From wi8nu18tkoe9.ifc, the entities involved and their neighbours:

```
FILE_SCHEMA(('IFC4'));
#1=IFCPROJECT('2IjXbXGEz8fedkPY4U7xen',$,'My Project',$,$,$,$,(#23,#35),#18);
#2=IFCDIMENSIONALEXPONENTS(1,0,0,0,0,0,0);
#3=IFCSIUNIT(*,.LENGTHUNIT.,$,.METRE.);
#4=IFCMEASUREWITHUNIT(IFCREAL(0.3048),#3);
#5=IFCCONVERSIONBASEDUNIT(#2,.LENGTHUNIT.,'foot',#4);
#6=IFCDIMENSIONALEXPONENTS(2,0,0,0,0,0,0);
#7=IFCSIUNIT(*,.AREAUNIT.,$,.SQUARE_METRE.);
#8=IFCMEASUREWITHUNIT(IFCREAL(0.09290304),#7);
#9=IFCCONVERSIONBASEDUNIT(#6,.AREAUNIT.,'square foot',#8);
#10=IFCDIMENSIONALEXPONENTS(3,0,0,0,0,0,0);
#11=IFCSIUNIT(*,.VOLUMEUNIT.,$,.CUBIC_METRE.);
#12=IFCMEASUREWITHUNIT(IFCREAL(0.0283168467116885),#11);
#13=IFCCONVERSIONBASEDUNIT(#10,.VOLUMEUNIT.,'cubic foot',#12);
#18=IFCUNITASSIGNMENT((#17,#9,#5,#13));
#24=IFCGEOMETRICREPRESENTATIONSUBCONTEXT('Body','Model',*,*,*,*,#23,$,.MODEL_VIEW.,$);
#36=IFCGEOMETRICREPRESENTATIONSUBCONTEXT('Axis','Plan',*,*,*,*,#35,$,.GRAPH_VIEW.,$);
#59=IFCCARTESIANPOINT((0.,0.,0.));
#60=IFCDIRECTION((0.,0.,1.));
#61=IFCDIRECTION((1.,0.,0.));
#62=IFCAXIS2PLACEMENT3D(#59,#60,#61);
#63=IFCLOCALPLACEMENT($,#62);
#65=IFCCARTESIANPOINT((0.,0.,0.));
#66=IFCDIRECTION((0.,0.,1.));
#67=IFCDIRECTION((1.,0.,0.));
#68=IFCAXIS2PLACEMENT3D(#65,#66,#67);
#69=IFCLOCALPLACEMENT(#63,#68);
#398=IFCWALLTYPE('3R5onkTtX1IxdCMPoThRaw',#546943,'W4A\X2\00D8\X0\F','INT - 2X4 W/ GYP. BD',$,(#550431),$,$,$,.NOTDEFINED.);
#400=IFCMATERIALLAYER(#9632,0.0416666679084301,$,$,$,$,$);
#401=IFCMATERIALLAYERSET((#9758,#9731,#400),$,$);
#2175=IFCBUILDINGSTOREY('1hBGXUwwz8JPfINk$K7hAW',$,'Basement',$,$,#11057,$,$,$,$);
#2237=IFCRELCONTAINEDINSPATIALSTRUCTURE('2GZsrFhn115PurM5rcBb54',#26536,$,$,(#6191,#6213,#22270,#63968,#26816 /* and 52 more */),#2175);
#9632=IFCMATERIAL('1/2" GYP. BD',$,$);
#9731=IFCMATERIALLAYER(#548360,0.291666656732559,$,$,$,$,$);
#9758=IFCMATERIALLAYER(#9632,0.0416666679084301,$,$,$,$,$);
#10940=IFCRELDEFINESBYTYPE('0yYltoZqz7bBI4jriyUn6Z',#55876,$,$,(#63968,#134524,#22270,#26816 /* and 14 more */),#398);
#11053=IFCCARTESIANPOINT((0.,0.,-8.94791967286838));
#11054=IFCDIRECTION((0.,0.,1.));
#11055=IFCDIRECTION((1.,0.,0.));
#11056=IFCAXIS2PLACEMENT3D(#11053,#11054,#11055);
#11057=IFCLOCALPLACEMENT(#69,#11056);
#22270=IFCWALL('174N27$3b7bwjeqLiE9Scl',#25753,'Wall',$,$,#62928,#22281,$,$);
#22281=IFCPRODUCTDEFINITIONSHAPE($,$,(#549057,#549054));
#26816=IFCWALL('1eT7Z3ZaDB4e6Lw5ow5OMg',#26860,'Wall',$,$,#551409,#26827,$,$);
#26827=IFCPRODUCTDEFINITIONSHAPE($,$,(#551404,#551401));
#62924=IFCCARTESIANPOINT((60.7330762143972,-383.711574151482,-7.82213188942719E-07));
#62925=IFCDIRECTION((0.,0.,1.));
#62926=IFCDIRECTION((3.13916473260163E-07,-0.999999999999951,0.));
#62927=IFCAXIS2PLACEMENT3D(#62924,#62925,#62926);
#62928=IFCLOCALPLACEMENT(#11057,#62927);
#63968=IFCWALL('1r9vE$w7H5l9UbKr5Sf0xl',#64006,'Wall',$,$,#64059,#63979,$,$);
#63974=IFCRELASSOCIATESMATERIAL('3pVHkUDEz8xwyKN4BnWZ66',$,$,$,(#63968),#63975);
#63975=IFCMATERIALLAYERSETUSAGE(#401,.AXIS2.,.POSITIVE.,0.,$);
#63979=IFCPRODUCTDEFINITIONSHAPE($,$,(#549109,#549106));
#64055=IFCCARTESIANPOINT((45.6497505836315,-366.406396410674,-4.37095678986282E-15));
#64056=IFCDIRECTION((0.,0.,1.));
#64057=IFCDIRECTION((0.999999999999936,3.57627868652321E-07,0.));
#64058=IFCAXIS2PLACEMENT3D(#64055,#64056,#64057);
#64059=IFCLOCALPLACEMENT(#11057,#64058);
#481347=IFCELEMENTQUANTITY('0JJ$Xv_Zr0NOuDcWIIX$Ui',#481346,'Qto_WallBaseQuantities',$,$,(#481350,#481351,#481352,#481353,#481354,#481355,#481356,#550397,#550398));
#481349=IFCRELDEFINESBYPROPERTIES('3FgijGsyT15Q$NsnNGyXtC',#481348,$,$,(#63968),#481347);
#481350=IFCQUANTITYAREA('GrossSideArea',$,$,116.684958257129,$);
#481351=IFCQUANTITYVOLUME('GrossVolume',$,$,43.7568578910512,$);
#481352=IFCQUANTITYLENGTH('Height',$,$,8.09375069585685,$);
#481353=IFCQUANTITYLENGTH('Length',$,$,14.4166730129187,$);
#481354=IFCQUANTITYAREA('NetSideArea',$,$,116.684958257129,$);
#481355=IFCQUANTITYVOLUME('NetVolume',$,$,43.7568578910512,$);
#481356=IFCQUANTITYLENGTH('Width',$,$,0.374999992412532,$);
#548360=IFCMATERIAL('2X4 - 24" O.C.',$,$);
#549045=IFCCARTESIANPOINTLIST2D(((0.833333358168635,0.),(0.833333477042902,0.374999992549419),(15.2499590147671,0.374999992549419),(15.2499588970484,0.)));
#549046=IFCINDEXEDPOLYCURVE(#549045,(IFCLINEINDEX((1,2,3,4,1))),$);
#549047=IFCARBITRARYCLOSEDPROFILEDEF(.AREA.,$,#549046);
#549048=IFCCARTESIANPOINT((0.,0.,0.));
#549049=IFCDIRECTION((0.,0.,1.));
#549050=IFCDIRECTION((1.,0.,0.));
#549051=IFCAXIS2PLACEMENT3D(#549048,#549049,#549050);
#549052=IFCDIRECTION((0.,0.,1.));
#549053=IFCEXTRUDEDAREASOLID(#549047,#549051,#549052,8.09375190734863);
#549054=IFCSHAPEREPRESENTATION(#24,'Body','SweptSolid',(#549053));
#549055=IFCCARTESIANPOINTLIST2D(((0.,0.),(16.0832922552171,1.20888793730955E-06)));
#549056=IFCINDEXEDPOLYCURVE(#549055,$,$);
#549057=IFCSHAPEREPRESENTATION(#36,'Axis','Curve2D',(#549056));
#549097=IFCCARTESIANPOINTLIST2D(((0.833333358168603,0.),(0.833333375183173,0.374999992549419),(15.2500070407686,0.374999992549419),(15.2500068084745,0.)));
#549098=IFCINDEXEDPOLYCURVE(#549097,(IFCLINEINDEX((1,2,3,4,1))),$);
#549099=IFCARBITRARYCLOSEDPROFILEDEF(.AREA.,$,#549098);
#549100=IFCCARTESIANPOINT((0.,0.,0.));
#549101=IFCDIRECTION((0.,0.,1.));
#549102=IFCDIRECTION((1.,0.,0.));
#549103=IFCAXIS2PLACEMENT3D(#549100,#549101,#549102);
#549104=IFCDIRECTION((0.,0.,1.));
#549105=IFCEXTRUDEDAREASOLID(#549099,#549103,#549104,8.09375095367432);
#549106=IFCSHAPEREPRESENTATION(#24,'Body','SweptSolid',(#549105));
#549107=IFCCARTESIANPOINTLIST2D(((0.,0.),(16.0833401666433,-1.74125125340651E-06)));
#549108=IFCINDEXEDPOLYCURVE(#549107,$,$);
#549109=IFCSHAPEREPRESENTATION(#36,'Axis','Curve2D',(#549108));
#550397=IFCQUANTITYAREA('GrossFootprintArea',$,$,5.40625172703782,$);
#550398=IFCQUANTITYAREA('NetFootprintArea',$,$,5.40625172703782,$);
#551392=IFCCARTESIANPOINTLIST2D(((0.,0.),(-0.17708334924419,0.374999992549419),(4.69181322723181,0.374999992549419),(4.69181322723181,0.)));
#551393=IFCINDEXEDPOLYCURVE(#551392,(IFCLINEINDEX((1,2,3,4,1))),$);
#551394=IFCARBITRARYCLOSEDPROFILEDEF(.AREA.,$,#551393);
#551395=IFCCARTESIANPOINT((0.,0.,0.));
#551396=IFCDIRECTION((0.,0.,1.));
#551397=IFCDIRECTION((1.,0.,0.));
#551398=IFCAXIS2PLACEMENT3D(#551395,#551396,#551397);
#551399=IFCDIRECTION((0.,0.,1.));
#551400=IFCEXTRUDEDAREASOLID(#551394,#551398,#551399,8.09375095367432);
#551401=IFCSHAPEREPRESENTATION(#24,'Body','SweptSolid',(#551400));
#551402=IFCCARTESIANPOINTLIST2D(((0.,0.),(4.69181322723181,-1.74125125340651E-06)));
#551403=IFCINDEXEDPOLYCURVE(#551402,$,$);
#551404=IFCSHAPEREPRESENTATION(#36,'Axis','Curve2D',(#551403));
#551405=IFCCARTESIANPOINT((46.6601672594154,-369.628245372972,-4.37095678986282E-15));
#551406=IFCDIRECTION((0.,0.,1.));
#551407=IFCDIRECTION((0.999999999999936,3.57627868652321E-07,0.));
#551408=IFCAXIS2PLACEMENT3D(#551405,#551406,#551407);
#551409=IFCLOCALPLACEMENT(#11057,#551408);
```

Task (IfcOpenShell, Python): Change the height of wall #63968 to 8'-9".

```python
import ifcopenshell
import ifcopenshell.api.pset
import ifcopenshell.geom
import ifcopenshell.util.element
import ifcopenshell.util.representation
import ifcopenshell.util.shape
import ifcopenshell.util.unit

model = ifcopenshell.open("wi8nu18tkoe9.ifc")
unit_scale = ifcopenshell.util.unit.calculate_unit_scale(model)
area_scale = ifcopenshell.util.unit.calculate_unit_scale(model, "AREAUNIT")
volume_scale = ifcopenshell.util.unit.calculate_unit_scale(model, "VOLUMEUNIT")
settings = ifcopenshell.geom.settings()


def volume(element):
    """Net volume in cubic metres, openings subtracted."""
    shape = ifcopenshell.geom.create_shape(settings, element)
    return ifcopenshell.util.shape.get_volume(shape.geometry)


wall = model.by_id(63968)
before = volume(wall)

body = ifcopenshell.util.representation.get_representation(wall, "Model", "Body")
solid = body.Items[0]
old_height = solid.Depth
solid.Depth = 105 * 0.0254 / unit_scale
after = volume(wall)
thickness = 0.1143  # wall thickness in metres

# Update the stored height, areas and volumes.
qto = model.by_id(ifcopenshell.util.element.get_pset(wall, "Qto_WallBaseQuantities", should_inherit=False)["id"])
ifcopenshell.api.pset.edit_qto(model, qto=qto, properties={
    "GrossSideArea": ifcopenshell.util.element.get_pset(wall, "Qto_WallBaseQuantities", "GrossSideArea") * solid.Depth / old_height,
    "GrossVolume": ifcopenshell.util.element.get_pset(wall, "Qto_WallBaseQuantities", "GrossVolume") * solid.Depth / old_height,
    "Height": solid.Depth,
    "NetSideArea": after / thickness / area_scale,
    "NetVolume": after / volume_scale,
})

print(f"height {old_height:g} -> {solid.Depth:g}, volume {before:.3f} -> {after:.3f} m3")

model.write("wi8nu18tkoe9_edited.ifc")
```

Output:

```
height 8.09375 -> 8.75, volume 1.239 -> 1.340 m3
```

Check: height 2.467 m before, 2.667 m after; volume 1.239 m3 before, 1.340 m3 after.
